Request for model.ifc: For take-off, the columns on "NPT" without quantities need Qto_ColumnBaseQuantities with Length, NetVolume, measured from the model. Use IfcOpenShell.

First a look at what the model holds.

```python
import ifcopenshell
import ifcopenshell.util.element
import ifcopenshell.util.unit

model = ifcopenshell.open("model.ifc")
print(model.schema)
for unit_type in ("LENGTHUNIT", "AREAUNIT", "VOLUMEUNIT"):
    print(unit_type, ifcopenshell.util.unit.calculate_unit_scale(model, unit_type))
storey = next(s for s in model.by_type("IfcBuildingStorey") if s.Name == "NPT")
columns = [e for e in ifcopenshell.util.element.get_decomposition(storey) if e.is_a("IfcColumn")]
for e in sorted(columns, key=lambda e: e.id()):
    print(e.id(), e.is_a(), e.Name, list(ifcopenshell.util.element.get_psets(e, qtos_only=True)), sep=" | ")
```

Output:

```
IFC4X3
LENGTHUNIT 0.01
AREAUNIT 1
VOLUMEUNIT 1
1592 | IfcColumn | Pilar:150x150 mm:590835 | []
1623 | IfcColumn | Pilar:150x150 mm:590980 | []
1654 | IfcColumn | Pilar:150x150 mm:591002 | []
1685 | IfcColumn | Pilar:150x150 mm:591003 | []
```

```python
import ifcopenshell
import ifcopenshell.api.pset
import ifcopenshell.geom
import ifcopenshell.util.element
import ifcopenshell.util.shape
import ifcopenshell.util.unit

model = ifcopenshell.open("model.ifc")
unit_scale = ifcopenshell.util.unit.calculate_unit_scale(model)
volume_scale = ifcopenshell.util.unit.calculate_unit_scale(model, "VOLUMEUNIT")
settings = ifcopenshell.geom.settings()

storey = next(s for s in model.by_type("IfcBuildingStorey") if s.Name == "NPT")
columns = [e for e in ifcopenshell.util.element.get_decomposition(storey) if e.is_a("IfcColumn")]

for e in sorted(columns, key=lambda e: e.id()):
    if ifcopenshell.util.element.get_psets(e, qtos_only=True, should_inherit=False):
        continue
    # Geometry comes back in metres, in the element's own axes.
    shape = ifcopenshell.geom.create_shape(settings, e)
    values = {
        "Length": ifcopenshell.util.shape.get_z(shape.geometry) / unit_scale,
        "NetVolume": ifcopenshell.util.shape.get_volume(shape.geometry) / volume_scale,
    }
    qto = ifcopenshell.api.pset.add_qto(model, product=e, name="Qto_ColumnBaseQuantities")
    ifcopenshell.api.pset.edit_qto(model, qto=qto, properties=values)
    print(e.id(), {k: round(v, 3) for k, v in values.items()})

model.write("model_v2.ifc")
```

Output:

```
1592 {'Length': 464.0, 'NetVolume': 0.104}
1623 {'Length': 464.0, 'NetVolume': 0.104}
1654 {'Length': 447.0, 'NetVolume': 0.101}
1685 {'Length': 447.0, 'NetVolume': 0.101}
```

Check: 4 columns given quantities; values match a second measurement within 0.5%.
